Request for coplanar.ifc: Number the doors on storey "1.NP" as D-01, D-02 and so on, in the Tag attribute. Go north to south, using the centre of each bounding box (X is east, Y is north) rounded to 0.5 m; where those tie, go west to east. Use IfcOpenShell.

First a look at what the model holds.

```python
import ifcopenshell
import ifcopenshell.util.element
import ifcopenshell.util.placement

model = ifcopenshell.open("coplanar.ifc")
print(model.schema)
storey = next(s for s in model.by_type("IfcBuildingStorey") if s.Name == "1.NP")
doors = [e for e in ifcopenshell.util.element.get_decomposition(storey) if e.is_a("IfcDoor")]
for e in sorted(doors, key=lambda e: e.id()):
    origin = ifcopenshell.util.placement.get_local_placement(e.ObjectPlacement)[:3, 3]
    print(e.id(), e.Tag, e.Name, origin.round(2) + 0.0, sep=" | ")
```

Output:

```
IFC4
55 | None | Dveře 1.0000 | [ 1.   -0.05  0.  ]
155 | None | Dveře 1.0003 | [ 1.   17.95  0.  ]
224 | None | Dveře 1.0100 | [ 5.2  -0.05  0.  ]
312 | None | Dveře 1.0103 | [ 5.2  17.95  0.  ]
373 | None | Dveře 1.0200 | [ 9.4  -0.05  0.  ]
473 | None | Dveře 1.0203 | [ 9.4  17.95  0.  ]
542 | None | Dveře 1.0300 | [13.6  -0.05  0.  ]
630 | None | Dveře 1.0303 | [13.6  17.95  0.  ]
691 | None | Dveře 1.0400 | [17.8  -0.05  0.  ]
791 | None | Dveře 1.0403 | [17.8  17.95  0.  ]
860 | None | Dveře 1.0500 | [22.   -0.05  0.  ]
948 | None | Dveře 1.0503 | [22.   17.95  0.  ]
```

```python
import ifcopenshell
import ifcopenshell.geom
import ifcopenshell.util.element
import ifcopenshell.util.shape

model = ifcopenshell.open("coplanar.ifc")
settings = ifcopenshell.geom.settings()
settings.set("use-world-coords", True)


def centre(element):
    shape = ifcopenshell.geom.create_shape(settings, element)
    return ifcopenshell.util.shape.get_bbox_centroid(shape.geometry)


storey = next(s for s in model.by_type("IfcBuildingStorey") if s.Name == "1.NP")
doors = [e for e in ifcopenshell.util.element.get_decomposition(storey) if e.is_a("IfcDoor")]

# Insertion points can sit at a corner or the storey origin, so sort by the geometry (in metres).
centres = {e: centre(e) for e in doors}
doors.sort(key=lambda e: (-round(centres[e][1] / 0.5), centres[e][0]))

for i, e in enumerate(doors, start=1):
    number = f"D-{i:02d}"
    e.Tag = number
    print(e.id(), number)

model.write("coplanar_v2.ifc")
```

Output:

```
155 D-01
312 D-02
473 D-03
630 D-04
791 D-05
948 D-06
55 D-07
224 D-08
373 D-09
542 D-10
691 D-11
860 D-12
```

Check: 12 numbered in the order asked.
